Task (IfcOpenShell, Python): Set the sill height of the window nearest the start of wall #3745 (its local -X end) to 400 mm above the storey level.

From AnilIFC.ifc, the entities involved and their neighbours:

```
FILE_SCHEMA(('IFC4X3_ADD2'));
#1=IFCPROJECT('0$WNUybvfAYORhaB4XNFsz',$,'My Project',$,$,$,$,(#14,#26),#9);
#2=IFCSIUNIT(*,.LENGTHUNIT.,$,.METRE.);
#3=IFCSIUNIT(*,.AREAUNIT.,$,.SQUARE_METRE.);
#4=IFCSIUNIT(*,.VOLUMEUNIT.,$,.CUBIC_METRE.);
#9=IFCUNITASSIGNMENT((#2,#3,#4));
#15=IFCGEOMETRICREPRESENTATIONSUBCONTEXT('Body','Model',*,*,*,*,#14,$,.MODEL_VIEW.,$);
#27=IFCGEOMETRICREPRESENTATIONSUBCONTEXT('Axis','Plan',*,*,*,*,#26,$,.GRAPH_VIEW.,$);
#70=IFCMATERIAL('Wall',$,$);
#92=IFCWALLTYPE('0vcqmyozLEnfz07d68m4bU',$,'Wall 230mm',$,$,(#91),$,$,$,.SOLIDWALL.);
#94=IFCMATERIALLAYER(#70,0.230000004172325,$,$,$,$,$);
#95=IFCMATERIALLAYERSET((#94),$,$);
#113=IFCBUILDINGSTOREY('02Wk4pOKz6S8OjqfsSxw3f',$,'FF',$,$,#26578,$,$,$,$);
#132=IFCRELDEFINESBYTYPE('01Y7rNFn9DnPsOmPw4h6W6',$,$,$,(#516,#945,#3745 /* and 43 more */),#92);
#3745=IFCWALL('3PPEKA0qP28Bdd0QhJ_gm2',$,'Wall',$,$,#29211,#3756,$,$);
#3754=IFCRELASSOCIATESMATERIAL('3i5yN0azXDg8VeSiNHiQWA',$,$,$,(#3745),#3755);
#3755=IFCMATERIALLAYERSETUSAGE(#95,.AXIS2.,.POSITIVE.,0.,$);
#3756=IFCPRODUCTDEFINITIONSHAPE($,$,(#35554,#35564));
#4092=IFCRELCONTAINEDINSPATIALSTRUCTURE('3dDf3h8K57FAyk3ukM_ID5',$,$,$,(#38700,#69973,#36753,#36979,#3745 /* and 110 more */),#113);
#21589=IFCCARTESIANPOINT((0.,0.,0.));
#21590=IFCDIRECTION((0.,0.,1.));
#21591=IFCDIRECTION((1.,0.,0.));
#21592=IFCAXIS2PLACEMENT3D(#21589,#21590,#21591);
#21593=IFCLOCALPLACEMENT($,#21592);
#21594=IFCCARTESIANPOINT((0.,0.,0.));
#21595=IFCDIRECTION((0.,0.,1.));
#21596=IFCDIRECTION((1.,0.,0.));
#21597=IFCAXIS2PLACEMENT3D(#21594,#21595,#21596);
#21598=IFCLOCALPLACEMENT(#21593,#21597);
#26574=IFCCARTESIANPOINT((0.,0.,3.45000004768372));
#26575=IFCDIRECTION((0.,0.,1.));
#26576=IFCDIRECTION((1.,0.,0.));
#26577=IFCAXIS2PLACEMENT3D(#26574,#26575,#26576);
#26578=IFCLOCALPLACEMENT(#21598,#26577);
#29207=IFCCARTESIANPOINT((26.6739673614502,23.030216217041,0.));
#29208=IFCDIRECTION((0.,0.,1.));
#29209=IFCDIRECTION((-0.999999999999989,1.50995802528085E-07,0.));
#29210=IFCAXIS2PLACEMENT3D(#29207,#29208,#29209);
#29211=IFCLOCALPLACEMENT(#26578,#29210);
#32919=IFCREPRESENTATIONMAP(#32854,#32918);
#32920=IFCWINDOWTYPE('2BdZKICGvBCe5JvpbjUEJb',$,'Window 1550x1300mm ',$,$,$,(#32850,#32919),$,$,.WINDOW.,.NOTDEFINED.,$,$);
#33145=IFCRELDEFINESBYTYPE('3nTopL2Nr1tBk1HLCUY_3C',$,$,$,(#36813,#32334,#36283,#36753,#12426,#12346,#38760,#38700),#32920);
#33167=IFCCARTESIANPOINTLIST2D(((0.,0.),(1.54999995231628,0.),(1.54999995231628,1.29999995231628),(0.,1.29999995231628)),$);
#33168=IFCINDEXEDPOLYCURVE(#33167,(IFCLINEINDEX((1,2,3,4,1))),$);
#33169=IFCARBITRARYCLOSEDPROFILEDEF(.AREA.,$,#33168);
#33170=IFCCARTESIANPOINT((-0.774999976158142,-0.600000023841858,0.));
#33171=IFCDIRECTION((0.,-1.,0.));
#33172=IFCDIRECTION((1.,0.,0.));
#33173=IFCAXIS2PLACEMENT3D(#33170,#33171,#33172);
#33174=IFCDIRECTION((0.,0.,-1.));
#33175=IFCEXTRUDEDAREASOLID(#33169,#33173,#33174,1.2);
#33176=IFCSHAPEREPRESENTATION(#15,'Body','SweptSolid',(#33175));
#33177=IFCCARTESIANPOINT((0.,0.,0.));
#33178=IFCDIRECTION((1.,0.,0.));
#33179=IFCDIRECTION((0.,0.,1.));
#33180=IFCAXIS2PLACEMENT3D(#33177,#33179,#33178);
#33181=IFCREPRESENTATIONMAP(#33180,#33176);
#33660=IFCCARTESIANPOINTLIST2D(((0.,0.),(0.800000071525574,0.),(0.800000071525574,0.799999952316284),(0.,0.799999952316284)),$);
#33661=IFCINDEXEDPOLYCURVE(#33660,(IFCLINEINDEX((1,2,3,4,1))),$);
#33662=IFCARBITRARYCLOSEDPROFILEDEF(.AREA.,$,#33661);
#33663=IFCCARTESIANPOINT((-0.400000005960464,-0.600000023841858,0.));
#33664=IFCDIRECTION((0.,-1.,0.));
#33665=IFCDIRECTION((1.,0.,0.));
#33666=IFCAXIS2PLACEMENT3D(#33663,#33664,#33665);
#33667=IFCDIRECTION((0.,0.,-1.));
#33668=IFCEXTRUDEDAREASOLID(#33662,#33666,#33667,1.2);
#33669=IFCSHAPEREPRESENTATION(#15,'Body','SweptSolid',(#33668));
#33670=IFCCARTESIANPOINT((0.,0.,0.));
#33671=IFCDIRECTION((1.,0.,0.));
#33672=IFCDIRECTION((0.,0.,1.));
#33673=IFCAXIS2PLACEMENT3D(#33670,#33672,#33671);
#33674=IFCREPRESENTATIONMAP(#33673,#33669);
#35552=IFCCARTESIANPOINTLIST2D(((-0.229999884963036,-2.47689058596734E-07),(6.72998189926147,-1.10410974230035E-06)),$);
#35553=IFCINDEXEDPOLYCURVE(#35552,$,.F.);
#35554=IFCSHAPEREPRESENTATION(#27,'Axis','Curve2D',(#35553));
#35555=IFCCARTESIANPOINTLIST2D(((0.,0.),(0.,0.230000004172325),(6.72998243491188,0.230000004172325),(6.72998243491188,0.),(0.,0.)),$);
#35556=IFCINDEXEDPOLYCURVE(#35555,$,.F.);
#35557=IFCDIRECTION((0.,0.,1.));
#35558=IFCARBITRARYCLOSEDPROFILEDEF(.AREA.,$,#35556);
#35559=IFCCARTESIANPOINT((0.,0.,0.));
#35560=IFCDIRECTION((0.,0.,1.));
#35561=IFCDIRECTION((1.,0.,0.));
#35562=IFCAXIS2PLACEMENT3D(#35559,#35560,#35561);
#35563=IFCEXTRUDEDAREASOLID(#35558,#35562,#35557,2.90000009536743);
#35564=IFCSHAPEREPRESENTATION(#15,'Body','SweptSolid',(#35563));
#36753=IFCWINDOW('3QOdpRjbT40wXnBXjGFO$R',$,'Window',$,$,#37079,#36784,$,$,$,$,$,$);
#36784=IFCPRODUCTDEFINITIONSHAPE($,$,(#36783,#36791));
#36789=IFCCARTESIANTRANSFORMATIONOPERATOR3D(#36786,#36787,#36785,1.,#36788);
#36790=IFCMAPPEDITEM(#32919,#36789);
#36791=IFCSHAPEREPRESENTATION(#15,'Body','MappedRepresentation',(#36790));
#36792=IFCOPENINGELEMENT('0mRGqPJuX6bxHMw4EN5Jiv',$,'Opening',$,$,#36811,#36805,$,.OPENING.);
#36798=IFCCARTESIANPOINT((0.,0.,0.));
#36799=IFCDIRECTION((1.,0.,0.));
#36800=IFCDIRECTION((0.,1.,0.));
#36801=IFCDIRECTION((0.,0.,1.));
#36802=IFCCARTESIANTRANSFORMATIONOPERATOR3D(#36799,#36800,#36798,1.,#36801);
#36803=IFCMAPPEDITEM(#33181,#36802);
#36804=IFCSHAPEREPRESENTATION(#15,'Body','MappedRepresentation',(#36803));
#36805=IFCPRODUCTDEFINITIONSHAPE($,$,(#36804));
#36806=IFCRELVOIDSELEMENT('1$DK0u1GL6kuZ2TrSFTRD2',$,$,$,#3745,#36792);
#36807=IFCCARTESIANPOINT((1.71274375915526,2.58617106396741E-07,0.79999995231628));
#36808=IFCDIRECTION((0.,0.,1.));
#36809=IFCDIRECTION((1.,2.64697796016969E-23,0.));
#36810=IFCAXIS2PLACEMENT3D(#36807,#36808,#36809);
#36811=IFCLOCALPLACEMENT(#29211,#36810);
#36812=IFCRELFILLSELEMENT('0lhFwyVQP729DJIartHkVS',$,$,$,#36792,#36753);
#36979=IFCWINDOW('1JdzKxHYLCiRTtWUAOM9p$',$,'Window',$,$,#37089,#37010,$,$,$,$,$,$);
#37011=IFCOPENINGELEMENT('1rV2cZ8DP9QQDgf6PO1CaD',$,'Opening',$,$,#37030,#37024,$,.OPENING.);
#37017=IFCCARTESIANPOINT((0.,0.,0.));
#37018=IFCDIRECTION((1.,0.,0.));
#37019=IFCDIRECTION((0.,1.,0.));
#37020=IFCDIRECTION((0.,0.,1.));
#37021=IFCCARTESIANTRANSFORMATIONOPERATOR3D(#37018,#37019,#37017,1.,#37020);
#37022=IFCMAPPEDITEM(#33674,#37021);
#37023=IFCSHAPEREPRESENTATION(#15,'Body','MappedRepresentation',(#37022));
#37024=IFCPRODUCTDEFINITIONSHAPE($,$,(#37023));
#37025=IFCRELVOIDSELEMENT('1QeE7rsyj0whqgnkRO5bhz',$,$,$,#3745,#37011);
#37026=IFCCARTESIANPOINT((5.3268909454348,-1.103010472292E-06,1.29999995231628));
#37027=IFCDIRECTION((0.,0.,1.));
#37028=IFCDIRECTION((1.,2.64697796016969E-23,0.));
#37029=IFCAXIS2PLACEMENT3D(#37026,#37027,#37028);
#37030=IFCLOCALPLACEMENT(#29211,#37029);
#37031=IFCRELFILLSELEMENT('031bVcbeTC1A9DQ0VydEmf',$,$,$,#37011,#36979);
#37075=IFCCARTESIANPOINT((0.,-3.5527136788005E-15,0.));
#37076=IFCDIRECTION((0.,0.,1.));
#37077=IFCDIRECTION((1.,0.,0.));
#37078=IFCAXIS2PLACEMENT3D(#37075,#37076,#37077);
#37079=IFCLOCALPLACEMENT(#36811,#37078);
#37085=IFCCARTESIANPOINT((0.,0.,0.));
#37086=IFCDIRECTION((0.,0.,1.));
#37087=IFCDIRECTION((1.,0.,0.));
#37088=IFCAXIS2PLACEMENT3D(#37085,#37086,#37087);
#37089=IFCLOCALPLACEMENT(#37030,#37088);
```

```python
import numpy as np
import ifcopenshell
import ifcopenshell.api.geometry
import ifcopenshell.geom
import ifcopenshell.util.element
import ifcopenshell.util.placement
import ifcopenshell.util.shape
import ifcopenshell.util.unit

model = ifcopenshell.open("AnilIFC.ifc")
unit_scale = ifcopenshell.util.unit.calculate_unit_scale(model)

window = model.by_id(36753)
opening = window.FillsVoids[0].RelatingOpeningElement
storey = ifcopenshell.util.element.get_container(window, ifc_class="IfcBuildingStorey")
level = ifcopenshell.util.placement.get_local_placement(storey.ObjectPlacement)[2, 3]

# The opening's origin need not be at the sill, so measure its lowest point.
shape = ifcopenshell.geom.create_shape(ifcopenshell.geom.settings(), opening)
bottom = ifcopenshell.util.shape.get_shape_bottom_elevation(shape, shape.geometry) / unit_scale
dz = level + 0.4 / unit_scale - bottom

shift = np.array([0.0, 0.0, dz])
# The window is placed relative to its opening, so it follows when the opening moves.
matrix = ifcopenshell.util.placement.get_local_placement(opening.ObjectPlacement)
matrix[:3, 3] += shift
ifcopenshell.api.geometry.edit_object_placement(
    model, product=opening, matrix=matrix, is_si=False, should_transform_children=True
)

print(f"moved by {dz * unit_scale:+.3f} m")

model.write("AnilIFC-out.ifc")
```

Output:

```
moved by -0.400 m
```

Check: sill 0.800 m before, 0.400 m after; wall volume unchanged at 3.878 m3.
